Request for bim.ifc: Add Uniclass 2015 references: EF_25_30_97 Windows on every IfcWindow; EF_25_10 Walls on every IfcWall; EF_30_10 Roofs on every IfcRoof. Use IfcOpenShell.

First a look at what the model holds.

```python
import ifcopenshell

model = ifcopenshell.open("bim.ifc")
print(model.schema)
print("classifications:", [c.Name for c in model.by_type("IfcClassification")])
for ifc_class in ("IfcDoor", "IfcRoof", "IfcStair", "IfcWall", "IfcWindow"):
    print(ifc_class, len(model.by_type(ifc_class)))
```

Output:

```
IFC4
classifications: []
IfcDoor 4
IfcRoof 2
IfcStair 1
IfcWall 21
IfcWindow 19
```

```python
import ifcopenshell
import ifcopenshell.api.classification

model = ifcopenshell.open("bim.ifc")

system = ifcopenshell.api.classification.add_classification(model, classification="Uniclass 2015")

codes = {
    "IfcWindow": ("EF_25_30_97", "Windows"),
    "IfcWall": ("EF_25_10", "Walls"),
    "IfcRoof": ("EF_30_10", "Roofs"),
}
for ifc_class, (code, name) in codes.items():
    products = model.by_type(ifc_class)
    ifcopenshell.api.classification.add_reference(
        model, products=products, classification=system, identification=code, name=name
    )
    print(code, len(products))

model.write("bim_rev.ifc")
```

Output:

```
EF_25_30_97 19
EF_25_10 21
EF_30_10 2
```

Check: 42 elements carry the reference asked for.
